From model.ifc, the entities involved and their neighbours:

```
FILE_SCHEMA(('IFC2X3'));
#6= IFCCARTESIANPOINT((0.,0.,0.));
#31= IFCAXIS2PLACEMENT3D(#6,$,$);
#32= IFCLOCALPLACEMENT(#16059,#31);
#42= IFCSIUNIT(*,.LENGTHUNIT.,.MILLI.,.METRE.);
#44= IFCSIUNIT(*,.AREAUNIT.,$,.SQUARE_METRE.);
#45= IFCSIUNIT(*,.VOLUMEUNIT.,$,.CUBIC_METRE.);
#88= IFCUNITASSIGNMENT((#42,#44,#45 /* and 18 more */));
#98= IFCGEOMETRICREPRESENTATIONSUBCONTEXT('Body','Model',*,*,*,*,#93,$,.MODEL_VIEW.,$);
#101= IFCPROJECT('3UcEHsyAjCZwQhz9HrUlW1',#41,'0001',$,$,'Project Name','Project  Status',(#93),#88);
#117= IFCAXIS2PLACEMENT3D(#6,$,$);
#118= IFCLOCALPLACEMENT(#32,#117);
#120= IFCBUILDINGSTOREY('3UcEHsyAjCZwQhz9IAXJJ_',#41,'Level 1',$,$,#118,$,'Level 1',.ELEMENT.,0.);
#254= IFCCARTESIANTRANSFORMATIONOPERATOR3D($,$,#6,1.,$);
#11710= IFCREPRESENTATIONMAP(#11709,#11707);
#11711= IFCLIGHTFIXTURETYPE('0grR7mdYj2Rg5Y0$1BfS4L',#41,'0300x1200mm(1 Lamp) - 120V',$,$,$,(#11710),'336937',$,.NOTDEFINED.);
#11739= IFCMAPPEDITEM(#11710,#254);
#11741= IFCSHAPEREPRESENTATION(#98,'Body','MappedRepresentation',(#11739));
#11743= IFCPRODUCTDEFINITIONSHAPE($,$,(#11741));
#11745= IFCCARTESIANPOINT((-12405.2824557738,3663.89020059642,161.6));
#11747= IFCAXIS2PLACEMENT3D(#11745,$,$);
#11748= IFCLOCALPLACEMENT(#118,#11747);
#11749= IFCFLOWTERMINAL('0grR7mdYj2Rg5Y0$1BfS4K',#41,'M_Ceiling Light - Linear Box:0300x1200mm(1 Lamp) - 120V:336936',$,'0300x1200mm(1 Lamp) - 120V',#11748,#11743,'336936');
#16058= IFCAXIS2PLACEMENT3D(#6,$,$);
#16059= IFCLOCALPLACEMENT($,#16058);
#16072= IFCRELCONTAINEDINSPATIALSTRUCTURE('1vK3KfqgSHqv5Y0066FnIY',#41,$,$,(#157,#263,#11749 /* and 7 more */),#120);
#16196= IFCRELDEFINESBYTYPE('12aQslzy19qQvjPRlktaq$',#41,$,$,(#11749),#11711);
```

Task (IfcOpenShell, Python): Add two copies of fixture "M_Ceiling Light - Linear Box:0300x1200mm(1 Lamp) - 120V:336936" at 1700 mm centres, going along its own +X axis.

```python
import ifcopenshell
import ifcopenshell.api.geometry
import ifcopenshell.api.root
import ifcopenshell.util.element
import ifcopenshell.util.placement
import ifcopenshell.util.unit

model = ifcopenshell.open("model.ifc")
unit_scale = ifcopenshell.util.unit.calculate_unit_scale(model)


def reuse_history(source, copy):
    """copy_class also copies each property set's owner history, people and application; keep the originals."""
    for rel in copy.IsDefinedBy:
        if rel.is_a("IfcRelDefinesByProperties") and (history := rel.RelatingPropertyDefinition.OwnerHistory):
            rel.RelatingPropertyDefinition.OwnerHistory = source.OwnerHistory
            ifcopenshell.util.element.remove_deep2(model, history)


source = model.by_guid("0grR7mdYj2Rg5Y0$1BfS4K")
base = ifcopenshell.util.placement.get_local_placement(source.ObjectPlacement)
step = base[:3, 0] * 1.7 / unit_scale

for i in range(1, 3):
    copy = ifcopenshell.api.root.copy_class(model, product=source)
    copy.Representation = ifcopenshell.util.element.copy_deep(
        model, source.Representation, exclude=["IfcGeometricRepresentationContext", "IfcRepresentationMap"]
    )
    copy.Name = "M_Ceiling Light - Linear Box:0300x1200mm(1 Lamp) - 120V"
    copy.Tag = None
    reuse_history(source, copy)
    matrix = base.copy()
    matrix[:3, 3] += i * step
    print("added at", matrix[:3, 3].round(3) + 0.0)
    ifcopenshell.api.geometry.edit_object_placement(model, product=copy, matrix=matrix, is_si=False)

model.write("model_edited.ifc")
```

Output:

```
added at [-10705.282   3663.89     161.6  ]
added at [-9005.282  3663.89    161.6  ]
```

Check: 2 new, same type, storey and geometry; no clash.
